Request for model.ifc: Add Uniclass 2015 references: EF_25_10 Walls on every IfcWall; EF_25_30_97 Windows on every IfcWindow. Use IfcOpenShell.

First a look at what the model holds.

```python
import ifcopenshell

model = ifcopenshell.open("model.ifc")
print(model.schema)
print("classifications:", [c.Name for c in model.by_type("IfcClassification")])
for ifc_class in ("IfcDoor", "IfcRoof", "IfcStair", "IfcWall", "IfcWindow"):
    print(ifc_class, len(model.by_type(ifc_class)))
```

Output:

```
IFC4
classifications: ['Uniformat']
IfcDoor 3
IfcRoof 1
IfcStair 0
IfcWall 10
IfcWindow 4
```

```python
import ifcopenshell
import ifcopenshell.api.classification

model = ifcopenshell.open("model.ifc")

system = ifcopenshell.api.classification.add_classification(model, classification="Uniclass 2015")

codes = {
    "IfcWall": ("EF_25_10", "Walls"),
    "IfcWindow": ("EF_25_30_97", "Windows"),
}
for ifc_class, (code, name) in codes.items():
    products = model.by_type(ifc_class)
    ifcopenshell.api.classification.add_reference(
        model, products=products, classification=system, identification=code, name=name
    )
    print(code, len(products))

model.write("model_updated.ifc")
```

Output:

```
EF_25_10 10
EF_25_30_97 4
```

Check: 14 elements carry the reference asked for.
